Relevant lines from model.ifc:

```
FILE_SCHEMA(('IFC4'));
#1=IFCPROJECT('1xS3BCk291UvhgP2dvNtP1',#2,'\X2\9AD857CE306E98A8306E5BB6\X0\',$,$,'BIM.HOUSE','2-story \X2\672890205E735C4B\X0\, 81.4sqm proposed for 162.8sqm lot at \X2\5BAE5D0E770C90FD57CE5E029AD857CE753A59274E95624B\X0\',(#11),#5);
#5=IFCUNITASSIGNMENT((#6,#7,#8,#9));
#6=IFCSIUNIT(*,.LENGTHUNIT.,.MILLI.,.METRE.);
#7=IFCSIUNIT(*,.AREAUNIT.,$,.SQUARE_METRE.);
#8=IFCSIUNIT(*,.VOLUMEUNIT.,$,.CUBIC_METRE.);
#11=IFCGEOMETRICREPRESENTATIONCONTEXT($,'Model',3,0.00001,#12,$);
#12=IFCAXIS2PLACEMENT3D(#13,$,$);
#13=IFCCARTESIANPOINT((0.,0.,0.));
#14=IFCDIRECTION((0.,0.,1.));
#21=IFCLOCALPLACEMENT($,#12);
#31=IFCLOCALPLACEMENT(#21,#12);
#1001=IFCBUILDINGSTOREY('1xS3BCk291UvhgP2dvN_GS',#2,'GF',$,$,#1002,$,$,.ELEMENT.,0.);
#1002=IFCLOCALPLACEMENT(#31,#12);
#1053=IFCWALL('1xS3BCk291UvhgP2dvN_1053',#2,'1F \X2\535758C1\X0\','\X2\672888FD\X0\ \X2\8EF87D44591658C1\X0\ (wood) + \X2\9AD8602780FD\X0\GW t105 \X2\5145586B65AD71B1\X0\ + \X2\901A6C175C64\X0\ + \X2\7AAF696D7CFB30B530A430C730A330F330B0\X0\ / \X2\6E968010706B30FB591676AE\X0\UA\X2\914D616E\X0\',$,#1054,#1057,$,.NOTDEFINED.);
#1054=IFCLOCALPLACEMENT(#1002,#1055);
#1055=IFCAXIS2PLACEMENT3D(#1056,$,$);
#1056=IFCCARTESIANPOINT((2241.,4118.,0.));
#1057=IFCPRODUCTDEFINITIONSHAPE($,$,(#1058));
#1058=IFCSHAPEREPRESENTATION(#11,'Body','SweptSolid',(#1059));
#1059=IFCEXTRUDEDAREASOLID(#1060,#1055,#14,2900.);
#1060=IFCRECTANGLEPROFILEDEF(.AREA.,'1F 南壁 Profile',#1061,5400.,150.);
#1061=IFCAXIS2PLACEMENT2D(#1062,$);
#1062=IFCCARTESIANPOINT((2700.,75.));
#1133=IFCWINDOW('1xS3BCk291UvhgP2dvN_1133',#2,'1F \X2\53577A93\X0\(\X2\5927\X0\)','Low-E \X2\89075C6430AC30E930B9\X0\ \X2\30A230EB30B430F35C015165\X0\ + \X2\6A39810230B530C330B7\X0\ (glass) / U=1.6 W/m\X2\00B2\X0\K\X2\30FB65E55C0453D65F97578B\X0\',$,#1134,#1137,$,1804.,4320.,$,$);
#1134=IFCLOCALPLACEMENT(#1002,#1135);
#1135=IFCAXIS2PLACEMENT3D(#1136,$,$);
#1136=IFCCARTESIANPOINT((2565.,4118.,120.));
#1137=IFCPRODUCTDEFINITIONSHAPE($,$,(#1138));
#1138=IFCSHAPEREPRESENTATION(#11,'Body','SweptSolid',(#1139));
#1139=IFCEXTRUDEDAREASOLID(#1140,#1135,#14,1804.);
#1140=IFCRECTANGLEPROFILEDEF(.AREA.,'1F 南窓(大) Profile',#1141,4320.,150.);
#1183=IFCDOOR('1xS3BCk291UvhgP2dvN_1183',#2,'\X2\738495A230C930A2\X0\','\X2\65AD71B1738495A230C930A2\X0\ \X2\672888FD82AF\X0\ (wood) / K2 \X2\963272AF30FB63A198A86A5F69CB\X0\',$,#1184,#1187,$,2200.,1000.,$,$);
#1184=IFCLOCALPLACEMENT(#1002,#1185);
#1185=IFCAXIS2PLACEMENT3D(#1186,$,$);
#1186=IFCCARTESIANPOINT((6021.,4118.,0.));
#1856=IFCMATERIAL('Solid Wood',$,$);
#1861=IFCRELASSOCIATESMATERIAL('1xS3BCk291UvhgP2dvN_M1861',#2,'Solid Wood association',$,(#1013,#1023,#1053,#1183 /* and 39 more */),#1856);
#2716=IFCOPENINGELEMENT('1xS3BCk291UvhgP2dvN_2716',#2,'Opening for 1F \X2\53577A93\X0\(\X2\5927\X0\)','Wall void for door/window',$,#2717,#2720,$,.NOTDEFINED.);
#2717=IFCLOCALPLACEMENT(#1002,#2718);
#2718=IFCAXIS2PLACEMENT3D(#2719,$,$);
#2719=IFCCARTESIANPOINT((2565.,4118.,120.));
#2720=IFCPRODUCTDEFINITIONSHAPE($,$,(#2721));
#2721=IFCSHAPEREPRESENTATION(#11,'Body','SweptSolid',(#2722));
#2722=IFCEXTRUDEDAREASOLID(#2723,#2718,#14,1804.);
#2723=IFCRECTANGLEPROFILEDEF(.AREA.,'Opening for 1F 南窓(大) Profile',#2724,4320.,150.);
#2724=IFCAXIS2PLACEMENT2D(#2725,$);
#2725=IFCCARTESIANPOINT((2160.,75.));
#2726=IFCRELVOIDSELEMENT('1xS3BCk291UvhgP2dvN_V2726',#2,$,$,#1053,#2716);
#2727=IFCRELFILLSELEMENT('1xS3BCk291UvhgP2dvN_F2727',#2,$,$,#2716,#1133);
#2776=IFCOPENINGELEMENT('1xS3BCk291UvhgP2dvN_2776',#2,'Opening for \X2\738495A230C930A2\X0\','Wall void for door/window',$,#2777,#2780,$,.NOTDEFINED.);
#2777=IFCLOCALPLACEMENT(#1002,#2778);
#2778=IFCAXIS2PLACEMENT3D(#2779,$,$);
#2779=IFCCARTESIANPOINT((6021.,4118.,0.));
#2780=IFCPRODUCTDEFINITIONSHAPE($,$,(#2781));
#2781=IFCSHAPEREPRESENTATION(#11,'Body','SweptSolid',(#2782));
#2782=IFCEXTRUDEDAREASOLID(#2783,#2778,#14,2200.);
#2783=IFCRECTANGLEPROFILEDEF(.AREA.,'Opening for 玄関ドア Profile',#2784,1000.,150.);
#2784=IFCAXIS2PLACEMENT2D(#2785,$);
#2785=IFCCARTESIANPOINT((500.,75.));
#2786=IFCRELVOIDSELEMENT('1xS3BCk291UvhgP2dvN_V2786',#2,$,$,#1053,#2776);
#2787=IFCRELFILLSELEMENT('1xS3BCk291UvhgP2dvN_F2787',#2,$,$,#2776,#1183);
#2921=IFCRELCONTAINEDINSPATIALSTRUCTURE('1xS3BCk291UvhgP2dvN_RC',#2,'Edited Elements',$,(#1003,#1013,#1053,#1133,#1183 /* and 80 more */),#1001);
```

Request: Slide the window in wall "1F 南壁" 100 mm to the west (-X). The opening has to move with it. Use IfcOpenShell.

```python
import ifcopenshell
import ifcopenshell.api.geometry
import ifcopenshell.util.placement
import ifcopenshell.util.unit

model = ifcopenshell.open("model.ifc")
unit_scale = ifcopenshell.util.unit.calculate_unit_scale(model)

window = model.by_id(1133)
opening = window.FillsVoids[0].RelatingOpeningElement
wall = opening.VoidsElements[0].RelatingBuildingElement

wall_matrix = ifcopenshell.util.placement.get_local_placement(wall.ObjectPlacement)
shift = wall_matrix[:3, 0] * -0.1 / unit_scale
before = ifcopenshell.util.placement.get_local_placement(window.ObjectPlacement)[:3, 3].copy()

# The window is not placed relative to its opening, so move both.
for product in (opening, window):
    matrix = ifcopenshell.util.placement.get_local_placement(product.ObjectPlacement)
    matrix[:3, 3] += shift
    ifcopenshell.api.geometry.edit_object_placement(model, product=product, matrix=matrix, is_si=False)

after = ifcopenshell.util.placement.get_local_placement(window.ObjectPlacement)[:3, 3]
print("window moved by", (after - before).round(3) + 0.0)

model.write("model_updated.ifc")
```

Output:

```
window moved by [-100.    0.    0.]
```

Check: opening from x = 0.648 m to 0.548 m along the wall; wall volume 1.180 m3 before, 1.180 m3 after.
